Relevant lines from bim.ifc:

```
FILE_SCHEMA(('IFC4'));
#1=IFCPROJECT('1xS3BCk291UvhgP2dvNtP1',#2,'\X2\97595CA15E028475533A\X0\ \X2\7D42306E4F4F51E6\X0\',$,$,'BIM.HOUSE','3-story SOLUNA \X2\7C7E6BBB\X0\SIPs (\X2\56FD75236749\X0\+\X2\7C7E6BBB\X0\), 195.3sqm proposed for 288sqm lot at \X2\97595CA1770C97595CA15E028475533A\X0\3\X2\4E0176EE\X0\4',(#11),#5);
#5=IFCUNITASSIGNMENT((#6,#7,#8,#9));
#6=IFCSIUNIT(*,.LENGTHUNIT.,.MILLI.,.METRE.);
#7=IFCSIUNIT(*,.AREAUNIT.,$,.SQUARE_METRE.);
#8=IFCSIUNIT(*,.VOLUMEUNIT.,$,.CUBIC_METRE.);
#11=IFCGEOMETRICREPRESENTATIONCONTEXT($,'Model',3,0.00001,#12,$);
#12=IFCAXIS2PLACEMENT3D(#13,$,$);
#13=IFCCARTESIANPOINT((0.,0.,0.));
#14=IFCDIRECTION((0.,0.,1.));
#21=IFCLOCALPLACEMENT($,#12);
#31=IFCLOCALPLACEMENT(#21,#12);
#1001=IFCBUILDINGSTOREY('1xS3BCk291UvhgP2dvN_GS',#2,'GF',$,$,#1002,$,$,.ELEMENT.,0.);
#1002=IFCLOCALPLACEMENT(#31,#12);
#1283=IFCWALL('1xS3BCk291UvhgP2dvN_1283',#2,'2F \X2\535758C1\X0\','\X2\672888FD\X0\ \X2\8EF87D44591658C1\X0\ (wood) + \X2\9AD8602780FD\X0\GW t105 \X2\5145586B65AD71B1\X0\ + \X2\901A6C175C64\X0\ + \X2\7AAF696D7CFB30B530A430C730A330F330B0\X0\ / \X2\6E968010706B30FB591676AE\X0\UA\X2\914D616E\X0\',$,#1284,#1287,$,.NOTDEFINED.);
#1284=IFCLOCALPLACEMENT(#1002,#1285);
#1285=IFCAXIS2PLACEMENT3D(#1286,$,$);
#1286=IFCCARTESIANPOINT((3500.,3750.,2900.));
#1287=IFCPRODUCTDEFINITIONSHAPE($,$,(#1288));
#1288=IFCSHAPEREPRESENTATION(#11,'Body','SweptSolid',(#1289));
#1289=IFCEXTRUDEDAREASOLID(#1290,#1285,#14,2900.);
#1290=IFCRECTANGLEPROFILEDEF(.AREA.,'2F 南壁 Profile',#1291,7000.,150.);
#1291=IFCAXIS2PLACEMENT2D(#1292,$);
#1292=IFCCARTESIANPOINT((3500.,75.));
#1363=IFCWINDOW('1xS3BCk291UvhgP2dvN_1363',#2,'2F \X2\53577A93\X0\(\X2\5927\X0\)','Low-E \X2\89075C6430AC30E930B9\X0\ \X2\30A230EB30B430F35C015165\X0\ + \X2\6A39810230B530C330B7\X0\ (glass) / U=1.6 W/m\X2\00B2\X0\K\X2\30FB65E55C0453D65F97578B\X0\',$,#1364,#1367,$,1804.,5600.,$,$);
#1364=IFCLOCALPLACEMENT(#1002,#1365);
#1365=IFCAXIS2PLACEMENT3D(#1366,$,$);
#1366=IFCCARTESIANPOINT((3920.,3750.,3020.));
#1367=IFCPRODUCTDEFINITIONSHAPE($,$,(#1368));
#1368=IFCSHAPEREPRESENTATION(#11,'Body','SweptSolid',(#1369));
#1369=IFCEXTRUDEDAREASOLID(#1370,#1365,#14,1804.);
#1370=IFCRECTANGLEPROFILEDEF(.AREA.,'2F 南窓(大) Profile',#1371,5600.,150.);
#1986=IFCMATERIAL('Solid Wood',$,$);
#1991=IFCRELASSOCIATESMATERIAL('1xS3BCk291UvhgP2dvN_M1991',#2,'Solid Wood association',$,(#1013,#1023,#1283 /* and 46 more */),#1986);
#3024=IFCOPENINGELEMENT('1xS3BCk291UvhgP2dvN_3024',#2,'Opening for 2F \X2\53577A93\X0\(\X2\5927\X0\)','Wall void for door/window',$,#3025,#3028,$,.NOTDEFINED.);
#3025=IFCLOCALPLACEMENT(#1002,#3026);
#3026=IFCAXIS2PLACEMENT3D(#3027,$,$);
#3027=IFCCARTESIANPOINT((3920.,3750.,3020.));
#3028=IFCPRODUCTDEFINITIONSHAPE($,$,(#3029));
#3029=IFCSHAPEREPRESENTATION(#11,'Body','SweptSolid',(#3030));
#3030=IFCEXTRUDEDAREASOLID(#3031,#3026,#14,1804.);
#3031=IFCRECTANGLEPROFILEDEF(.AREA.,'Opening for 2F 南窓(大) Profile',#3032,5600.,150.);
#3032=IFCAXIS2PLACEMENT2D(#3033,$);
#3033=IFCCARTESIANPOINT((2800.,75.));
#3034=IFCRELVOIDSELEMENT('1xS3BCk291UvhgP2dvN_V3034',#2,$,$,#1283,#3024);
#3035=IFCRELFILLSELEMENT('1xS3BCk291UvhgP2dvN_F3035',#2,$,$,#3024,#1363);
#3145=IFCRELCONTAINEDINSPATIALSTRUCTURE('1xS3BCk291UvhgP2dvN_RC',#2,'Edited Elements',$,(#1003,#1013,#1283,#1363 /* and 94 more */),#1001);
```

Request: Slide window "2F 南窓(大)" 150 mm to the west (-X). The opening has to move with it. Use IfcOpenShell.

```python
import ifcopenshell
import ifcopenshell.api.geometry
import ifcopenshell.util.placement

model = ifcopenshell.open("bim.ifc")

window = model.by_guid("1xS3BCk291UvhgP2dvN_1363")
opening = window.FillsVoids[0].RelatingOpeningElement
wall = opening.VoidsElements[0].RelatingBuildingElement

wall_matrix = ifcopenshell.util.placement.get_local_placement(wall.ObjectPlacement)
shift = wall_matrix[:3, 0] * -150.0
before = ifcopenshell.util.placement.get_local_placement(window.ObjectPlacement)[:3, 3].copy()

# The window is not placed relative to its opening, so move both.
for product in (opening, window):
    matrix = ifcopenshell.util.placement.get_local_placement(product.ObjectPlacement)
    matrix[:3, 3] += shift
    ifcopenshell.api.geometry.edit_object_placement(model, product=product, matrix=matrix, is_si=False)

after = ifcopenshell.util.placement.get_local_placement(window.ObjectPlacement)[:3, 3]
print("window moved by", (after - before).round(3) + 0.0)

model.write("bim_rev.ifc")
```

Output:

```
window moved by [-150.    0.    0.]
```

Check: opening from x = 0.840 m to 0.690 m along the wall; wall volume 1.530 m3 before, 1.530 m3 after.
